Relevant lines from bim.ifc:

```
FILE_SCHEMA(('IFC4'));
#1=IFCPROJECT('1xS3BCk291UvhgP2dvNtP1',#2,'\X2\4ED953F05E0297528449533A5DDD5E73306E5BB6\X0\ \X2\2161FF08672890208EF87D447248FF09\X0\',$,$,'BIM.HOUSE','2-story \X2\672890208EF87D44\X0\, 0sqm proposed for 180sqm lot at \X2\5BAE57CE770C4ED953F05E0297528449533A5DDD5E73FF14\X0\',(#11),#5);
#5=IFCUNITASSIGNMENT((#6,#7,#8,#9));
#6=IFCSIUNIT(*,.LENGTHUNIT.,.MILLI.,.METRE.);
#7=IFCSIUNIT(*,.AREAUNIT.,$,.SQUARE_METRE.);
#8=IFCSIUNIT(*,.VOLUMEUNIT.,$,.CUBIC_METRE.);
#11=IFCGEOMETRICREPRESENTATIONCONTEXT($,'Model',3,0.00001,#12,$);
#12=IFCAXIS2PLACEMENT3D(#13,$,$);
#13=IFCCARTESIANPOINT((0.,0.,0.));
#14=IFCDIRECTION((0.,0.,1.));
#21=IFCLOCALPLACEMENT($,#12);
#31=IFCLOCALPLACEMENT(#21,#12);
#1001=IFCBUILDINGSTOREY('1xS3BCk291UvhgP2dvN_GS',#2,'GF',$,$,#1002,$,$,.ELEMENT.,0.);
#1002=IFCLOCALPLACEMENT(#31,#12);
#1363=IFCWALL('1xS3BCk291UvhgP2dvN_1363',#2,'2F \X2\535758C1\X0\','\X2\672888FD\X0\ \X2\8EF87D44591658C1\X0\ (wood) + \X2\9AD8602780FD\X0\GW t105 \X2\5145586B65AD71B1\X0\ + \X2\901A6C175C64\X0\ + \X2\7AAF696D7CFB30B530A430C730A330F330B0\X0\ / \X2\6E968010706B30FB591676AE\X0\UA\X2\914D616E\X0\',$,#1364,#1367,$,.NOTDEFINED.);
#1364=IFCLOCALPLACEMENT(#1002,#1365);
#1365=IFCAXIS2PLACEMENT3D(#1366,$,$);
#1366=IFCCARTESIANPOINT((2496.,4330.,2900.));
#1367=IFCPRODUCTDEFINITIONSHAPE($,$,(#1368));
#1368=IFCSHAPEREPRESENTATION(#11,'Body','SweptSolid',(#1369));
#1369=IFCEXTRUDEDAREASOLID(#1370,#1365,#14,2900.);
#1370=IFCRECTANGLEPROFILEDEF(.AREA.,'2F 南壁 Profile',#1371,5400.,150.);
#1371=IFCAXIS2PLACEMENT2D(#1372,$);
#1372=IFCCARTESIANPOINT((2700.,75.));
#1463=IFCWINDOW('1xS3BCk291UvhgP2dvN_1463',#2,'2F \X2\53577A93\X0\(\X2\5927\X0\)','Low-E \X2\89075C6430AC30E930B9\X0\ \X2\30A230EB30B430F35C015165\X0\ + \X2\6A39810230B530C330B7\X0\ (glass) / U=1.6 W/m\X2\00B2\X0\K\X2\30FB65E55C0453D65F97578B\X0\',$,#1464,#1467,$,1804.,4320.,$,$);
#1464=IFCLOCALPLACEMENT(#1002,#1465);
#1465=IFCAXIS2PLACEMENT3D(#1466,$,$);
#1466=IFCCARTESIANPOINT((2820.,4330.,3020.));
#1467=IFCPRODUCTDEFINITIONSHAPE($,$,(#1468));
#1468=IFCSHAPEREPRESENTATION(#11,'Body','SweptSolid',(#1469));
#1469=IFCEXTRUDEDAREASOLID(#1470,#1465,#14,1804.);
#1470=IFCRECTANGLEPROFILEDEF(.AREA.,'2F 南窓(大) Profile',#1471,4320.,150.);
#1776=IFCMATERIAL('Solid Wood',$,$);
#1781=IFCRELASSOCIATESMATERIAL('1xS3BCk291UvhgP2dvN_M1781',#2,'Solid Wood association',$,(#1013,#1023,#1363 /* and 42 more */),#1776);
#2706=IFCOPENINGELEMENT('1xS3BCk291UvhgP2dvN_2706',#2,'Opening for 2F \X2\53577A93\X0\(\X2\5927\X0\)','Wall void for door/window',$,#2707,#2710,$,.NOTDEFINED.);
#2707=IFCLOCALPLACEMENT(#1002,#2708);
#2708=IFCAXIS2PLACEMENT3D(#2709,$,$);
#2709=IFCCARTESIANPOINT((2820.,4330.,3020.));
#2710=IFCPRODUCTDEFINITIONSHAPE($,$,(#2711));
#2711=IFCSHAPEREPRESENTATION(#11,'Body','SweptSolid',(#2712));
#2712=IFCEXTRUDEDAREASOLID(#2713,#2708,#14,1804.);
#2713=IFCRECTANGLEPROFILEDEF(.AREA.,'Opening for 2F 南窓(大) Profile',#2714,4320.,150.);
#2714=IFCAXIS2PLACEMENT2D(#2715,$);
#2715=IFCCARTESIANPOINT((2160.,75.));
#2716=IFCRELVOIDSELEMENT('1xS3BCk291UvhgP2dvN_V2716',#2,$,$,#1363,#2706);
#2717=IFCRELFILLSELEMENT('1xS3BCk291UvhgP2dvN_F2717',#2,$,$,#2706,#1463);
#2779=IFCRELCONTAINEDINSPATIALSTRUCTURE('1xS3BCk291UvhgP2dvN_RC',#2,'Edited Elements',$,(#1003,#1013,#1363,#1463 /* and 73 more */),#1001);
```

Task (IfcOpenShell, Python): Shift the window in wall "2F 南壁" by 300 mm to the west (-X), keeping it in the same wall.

```python
import ifcopenshell
import ifcopenshell.api.geometry
import ifcopenshell.util.placement
import ifcopenshell.util.unit

model = ifcopenshell.open("bim.ifc")
unit_scale = ifcopenshell.util.unit.calculate_unit_scale(model)

window = model.by_guid("1xS3BCk291UvhgP2dvN_1463")
opening = window.FillsVoids[0].RelatingOpeningElement
wall = opening.VoidsElements[0].RelatingBuildingElement

wall_matrix = ifcopenshell.util.placement.get_local_placement(wall.ObjectPlacement)
shift = wall_matrix[:3, 0] * -0.3 / unit_scale
before = ifcopenshell.util.placement.get_local_placement(window.ObjectPlacement)[:3, 3].copy()

# The window is not placed relative to its opening, so move both.
for product in (opening, window):
    matrix = ifcopenshell.util.placement.get_local_placement(product.ObjectPlacement)
    matrix[:3, 3] += shift
    ifcopenshell.api.geometry.edit_object_placement(model, product=product, matrix=matrix, is_si=False)

after = ifcopenshell.util.placement.get_local_placement(window.ObjectPlacement)[:3, 3]
print("window moved by", (after - before).round(3) + 0.0)

model.write("bim_rev.ifc")
```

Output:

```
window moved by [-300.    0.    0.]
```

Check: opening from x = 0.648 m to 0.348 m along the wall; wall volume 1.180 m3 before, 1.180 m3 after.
